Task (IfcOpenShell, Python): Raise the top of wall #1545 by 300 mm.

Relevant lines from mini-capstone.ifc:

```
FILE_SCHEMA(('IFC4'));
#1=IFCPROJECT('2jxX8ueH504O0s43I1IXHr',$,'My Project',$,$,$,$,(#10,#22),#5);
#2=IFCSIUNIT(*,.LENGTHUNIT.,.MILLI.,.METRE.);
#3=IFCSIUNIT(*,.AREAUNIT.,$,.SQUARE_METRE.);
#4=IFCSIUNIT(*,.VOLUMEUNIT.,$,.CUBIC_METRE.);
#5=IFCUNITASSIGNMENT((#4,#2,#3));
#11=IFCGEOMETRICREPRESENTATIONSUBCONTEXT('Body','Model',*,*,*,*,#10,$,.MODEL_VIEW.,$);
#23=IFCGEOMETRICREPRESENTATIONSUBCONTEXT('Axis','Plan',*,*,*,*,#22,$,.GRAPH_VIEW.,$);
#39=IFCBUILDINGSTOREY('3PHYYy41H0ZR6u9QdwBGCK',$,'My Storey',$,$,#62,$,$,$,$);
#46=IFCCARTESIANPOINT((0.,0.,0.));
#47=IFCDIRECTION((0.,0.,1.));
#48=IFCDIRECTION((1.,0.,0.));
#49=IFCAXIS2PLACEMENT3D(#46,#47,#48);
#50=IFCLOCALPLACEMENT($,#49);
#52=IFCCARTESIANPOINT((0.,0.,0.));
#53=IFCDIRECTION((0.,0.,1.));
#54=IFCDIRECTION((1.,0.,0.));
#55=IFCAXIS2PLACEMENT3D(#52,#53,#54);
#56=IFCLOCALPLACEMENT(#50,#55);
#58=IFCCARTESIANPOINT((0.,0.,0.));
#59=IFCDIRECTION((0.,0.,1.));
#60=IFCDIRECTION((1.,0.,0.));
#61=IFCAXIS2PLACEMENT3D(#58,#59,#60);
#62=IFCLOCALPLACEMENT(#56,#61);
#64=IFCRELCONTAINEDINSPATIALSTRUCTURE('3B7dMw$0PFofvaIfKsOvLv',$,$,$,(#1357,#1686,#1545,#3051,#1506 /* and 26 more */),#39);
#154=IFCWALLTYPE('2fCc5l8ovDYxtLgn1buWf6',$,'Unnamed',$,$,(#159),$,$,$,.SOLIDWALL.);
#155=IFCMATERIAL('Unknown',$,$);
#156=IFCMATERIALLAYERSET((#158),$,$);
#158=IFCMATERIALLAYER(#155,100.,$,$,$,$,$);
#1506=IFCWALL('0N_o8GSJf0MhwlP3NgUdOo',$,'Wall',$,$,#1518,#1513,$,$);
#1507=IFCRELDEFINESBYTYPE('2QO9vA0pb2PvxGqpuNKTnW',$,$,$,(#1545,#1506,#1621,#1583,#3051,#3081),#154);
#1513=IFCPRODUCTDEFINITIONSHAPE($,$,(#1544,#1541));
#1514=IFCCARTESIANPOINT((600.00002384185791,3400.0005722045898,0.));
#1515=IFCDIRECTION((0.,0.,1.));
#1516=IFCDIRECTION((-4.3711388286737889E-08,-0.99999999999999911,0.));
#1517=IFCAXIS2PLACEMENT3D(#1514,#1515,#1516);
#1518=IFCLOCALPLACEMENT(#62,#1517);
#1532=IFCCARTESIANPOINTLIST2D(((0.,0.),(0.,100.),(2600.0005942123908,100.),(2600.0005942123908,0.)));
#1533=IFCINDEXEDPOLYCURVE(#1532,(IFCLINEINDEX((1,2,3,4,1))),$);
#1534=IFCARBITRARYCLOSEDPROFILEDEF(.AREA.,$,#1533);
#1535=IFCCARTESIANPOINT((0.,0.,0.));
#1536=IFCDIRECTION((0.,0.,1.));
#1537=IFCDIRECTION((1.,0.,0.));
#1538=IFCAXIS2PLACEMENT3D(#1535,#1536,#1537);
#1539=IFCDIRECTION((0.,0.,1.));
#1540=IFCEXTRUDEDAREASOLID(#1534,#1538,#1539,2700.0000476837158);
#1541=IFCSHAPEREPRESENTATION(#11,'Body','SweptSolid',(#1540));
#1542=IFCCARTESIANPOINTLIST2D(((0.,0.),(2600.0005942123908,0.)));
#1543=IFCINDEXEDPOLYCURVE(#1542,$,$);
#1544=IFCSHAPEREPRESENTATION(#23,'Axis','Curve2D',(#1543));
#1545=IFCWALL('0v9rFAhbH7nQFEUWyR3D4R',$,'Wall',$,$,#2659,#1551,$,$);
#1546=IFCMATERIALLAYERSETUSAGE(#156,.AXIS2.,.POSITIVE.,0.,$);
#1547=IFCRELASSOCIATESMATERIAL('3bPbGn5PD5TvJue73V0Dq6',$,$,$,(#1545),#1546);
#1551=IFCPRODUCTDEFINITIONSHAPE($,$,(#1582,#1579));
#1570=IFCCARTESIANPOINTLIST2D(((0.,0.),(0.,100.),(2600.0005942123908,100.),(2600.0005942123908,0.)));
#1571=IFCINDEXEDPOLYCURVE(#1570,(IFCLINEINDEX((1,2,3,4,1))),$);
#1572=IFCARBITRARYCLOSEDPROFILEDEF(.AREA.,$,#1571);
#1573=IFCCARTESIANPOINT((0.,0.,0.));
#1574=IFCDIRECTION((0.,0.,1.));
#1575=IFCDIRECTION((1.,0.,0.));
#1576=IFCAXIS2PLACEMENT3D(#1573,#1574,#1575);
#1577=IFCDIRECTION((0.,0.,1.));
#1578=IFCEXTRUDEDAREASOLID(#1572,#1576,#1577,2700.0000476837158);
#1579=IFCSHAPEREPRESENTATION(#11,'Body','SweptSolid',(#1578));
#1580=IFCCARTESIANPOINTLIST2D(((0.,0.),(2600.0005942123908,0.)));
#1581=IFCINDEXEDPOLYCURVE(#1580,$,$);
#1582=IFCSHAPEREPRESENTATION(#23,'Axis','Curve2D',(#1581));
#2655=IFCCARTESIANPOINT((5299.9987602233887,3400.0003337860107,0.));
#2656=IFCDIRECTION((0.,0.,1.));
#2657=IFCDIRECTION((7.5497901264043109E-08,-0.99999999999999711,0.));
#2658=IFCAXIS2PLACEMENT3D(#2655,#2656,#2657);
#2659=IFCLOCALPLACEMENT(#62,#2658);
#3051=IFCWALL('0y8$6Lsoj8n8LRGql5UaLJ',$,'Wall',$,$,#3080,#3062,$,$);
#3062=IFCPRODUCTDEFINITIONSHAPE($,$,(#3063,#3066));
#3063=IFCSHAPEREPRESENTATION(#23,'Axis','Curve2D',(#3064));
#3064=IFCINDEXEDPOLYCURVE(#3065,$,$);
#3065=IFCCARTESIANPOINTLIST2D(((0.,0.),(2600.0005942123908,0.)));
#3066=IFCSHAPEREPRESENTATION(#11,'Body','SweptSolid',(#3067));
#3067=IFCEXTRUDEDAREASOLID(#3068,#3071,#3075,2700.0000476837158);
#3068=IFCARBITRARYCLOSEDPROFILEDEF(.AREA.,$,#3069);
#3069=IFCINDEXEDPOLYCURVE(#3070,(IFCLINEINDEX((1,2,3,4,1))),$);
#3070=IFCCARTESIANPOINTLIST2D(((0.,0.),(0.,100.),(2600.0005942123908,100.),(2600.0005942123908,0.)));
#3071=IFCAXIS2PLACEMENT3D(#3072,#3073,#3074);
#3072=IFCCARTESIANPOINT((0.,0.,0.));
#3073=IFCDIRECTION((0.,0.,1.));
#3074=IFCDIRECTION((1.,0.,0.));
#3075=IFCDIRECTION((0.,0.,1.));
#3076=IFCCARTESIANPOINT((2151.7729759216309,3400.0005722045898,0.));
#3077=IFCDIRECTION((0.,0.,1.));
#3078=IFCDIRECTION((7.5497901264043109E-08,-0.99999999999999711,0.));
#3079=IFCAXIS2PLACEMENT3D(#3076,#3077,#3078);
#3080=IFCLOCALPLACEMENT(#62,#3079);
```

```python
import ifcopenshell
import ifcopenshell.geom
import ifcopenshell.util.representation
import ifcopenshell.util.shape

model = ifcopenshell.open("mini-capstone.ifc")
settings = ifcopenshell.geom.settings()


def volume(element):
    """Net volume in cubic metres, openings subtracted."""
    shape = ifcopenshell.geom.create_shape(settings, element)
    return ifcopenshell.util.shape.get_volume(shape.geometry)


wall = model.by_id(1545)
before = volume(wall)

body = ifcopenshell.util.representation.get_representation(wall, "Model", "Body")
solid = body.Items[0]
old_height = solid.Depth
solid.Depth += 300.0
after = volume(wall)

print(f"height {old_height:g} -> {solid.Depth:g}, volume {before:.3f} -> {after:.3f} m3")

model.write("mini-capstone-out.ifc")
```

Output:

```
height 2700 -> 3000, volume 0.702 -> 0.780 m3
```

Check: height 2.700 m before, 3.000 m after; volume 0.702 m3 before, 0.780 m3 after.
